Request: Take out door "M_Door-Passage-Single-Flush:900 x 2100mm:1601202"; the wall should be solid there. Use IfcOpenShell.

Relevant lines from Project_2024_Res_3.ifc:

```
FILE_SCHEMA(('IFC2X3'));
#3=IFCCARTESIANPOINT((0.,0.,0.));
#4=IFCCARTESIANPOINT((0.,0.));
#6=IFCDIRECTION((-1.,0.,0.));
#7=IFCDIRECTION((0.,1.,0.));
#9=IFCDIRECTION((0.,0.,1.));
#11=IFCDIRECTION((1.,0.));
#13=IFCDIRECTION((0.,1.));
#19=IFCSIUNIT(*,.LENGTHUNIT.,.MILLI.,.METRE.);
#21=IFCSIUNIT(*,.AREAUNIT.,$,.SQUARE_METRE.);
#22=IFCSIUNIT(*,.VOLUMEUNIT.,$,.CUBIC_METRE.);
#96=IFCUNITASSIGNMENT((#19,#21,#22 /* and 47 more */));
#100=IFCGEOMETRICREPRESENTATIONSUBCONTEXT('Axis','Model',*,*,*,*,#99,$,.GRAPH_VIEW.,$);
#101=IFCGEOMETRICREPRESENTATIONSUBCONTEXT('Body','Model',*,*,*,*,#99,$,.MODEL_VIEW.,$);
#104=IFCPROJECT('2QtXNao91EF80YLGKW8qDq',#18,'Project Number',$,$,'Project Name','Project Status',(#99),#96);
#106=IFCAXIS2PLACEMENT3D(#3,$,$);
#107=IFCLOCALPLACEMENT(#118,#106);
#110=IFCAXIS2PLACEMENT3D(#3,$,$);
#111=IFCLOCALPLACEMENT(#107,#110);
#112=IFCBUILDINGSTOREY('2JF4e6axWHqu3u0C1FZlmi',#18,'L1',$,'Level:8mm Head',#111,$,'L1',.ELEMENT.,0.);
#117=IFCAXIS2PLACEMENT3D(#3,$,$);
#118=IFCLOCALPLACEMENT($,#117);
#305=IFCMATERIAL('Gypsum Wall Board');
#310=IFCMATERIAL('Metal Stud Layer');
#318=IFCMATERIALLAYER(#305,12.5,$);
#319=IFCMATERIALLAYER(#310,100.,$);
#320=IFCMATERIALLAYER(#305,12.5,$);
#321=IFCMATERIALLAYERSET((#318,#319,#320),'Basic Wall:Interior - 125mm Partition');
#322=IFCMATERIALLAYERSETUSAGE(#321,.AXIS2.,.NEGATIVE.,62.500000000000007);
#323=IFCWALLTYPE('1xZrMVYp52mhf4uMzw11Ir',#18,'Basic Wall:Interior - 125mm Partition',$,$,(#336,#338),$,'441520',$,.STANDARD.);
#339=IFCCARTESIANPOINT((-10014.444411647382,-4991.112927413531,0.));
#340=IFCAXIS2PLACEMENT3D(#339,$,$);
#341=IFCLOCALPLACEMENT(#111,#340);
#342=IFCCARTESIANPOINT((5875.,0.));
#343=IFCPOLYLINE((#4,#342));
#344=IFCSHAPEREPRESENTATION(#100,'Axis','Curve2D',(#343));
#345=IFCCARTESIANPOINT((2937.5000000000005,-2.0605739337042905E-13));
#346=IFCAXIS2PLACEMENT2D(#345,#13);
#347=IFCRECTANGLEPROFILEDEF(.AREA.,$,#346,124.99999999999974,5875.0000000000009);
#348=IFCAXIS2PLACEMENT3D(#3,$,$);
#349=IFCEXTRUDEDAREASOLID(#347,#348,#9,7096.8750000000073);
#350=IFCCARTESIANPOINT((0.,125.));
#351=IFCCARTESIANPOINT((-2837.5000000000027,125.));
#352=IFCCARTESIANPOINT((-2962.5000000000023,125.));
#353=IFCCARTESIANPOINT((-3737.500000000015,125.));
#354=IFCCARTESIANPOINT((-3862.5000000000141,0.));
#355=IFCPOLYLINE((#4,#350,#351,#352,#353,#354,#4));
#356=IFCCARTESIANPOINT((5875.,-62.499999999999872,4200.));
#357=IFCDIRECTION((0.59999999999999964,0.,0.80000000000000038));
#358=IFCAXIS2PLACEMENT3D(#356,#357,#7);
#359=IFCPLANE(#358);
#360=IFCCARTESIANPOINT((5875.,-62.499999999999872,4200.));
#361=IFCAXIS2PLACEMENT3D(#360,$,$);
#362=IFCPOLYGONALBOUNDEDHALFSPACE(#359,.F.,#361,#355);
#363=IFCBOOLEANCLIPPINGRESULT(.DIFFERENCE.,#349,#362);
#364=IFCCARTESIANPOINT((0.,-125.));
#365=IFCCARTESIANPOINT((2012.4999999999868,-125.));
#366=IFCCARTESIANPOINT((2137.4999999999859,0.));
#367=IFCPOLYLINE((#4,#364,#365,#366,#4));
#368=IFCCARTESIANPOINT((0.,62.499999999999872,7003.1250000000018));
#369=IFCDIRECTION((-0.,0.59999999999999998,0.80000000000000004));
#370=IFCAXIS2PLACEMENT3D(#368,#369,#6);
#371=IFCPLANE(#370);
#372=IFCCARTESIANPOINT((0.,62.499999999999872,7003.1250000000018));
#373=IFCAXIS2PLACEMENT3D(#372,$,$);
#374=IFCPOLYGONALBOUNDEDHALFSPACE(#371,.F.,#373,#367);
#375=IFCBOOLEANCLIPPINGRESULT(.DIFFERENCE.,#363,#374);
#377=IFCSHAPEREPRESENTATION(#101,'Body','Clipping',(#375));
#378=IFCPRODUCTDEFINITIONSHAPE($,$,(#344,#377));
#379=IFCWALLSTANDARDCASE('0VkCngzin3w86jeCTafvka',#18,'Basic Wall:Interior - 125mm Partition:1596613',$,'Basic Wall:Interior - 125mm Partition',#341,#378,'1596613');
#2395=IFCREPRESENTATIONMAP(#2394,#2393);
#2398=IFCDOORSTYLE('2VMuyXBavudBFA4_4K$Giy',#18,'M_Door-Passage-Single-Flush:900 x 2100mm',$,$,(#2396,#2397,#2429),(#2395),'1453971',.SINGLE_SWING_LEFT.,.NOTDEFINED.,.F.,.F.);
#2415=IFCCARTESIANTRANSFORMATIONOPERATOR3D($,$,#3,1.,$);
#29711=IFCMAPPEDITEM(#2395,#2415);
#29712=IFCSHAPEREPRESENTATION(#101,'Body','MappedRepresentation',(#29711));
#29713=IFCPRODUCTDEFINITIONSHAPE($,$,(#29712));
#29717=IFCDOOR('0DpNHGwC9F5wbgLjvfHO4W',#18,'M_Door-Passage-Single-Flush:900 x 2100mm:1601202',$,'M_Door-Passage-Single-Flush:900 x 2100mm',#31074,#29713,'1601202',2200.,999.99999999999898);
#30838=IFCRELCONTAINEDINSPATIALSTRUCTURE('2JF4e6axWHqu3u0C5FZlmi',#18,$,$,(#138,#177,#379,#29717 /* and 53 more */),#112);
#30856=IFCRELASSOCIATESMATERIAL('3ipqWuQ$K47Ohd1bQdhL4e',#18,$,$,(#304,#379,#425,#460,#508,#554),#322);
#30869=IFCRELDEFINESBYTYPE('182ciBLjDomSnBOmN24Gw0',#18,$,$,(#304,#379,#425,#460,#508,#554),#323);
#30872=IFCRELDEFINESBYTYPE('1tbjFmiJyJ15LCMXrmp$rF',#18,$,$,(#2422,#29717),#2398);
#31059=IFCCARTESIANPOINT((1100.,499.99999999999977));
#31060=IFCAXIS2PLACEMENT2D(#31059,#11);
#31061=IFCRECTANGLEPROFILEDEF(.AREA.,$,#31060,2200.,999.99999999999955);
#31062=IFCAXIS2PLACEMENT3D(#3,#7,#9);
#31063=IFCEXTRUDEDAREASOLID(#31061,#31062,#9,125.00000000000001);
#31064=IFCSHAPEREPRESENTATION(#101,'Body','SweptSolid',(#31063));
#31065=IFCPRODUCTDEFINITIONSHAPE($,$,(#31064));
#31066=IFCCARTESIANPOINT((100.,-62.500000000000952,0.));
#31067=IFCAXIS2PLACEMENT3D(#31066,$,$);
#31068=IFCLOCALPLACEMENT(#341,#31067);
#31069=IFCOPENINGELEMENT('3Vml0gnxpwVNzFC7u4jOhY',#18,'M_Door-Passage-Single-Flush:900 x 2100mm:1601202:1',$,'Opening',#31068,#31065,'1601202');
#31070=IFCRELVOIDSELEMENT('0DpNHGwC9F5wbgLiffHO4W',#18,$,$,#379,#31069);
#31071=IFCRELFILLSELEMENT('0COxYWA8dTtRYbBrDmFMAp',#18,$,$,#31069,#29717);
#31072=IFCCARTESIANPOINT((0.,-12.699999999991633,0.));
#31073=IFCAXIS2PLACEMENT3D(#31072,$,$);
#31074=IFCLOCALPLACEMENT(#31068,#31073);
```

```python
import ifcopenshell
import ifcopenshell.api.feature
import ifcopenshell.api.root
import ifcopenshell.geom
import ifcopenshell.util.shape

model = ifcopenshell.open("Project_2024_Res_3.ifc")
settings = ifcopenshell.geom.settings()


def volume(element):
    """Net volume in cubic metres, openings subtracted."""
    shape = ifcopenshell.geom.create_shape(settings, element)
    return ifcopenshell.util.shape.get_volume(shape.geometry)


door = model.by_guid("0DpNHGwC9F5wbgLjvfHO4W")
opening = door.FillsVoids[0].RelatingOpeningElement
wall = opening.VoidsElements[0].RelatingBuildingElement
before = volume(wall)

ifcopenshell.api.root.remove_product(model, product=door)
ifcopenshell.api.feature.remove_feature(model, feature=opening)

after = volume(wall)

print(f"wall volume {before:.3f} -> {after:.3f} m3")

model.write("Project_2024_Res_3_edited.ifc")
```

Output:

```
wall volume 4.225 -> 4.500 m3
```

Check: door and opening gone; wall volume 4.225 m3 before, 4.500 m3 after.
